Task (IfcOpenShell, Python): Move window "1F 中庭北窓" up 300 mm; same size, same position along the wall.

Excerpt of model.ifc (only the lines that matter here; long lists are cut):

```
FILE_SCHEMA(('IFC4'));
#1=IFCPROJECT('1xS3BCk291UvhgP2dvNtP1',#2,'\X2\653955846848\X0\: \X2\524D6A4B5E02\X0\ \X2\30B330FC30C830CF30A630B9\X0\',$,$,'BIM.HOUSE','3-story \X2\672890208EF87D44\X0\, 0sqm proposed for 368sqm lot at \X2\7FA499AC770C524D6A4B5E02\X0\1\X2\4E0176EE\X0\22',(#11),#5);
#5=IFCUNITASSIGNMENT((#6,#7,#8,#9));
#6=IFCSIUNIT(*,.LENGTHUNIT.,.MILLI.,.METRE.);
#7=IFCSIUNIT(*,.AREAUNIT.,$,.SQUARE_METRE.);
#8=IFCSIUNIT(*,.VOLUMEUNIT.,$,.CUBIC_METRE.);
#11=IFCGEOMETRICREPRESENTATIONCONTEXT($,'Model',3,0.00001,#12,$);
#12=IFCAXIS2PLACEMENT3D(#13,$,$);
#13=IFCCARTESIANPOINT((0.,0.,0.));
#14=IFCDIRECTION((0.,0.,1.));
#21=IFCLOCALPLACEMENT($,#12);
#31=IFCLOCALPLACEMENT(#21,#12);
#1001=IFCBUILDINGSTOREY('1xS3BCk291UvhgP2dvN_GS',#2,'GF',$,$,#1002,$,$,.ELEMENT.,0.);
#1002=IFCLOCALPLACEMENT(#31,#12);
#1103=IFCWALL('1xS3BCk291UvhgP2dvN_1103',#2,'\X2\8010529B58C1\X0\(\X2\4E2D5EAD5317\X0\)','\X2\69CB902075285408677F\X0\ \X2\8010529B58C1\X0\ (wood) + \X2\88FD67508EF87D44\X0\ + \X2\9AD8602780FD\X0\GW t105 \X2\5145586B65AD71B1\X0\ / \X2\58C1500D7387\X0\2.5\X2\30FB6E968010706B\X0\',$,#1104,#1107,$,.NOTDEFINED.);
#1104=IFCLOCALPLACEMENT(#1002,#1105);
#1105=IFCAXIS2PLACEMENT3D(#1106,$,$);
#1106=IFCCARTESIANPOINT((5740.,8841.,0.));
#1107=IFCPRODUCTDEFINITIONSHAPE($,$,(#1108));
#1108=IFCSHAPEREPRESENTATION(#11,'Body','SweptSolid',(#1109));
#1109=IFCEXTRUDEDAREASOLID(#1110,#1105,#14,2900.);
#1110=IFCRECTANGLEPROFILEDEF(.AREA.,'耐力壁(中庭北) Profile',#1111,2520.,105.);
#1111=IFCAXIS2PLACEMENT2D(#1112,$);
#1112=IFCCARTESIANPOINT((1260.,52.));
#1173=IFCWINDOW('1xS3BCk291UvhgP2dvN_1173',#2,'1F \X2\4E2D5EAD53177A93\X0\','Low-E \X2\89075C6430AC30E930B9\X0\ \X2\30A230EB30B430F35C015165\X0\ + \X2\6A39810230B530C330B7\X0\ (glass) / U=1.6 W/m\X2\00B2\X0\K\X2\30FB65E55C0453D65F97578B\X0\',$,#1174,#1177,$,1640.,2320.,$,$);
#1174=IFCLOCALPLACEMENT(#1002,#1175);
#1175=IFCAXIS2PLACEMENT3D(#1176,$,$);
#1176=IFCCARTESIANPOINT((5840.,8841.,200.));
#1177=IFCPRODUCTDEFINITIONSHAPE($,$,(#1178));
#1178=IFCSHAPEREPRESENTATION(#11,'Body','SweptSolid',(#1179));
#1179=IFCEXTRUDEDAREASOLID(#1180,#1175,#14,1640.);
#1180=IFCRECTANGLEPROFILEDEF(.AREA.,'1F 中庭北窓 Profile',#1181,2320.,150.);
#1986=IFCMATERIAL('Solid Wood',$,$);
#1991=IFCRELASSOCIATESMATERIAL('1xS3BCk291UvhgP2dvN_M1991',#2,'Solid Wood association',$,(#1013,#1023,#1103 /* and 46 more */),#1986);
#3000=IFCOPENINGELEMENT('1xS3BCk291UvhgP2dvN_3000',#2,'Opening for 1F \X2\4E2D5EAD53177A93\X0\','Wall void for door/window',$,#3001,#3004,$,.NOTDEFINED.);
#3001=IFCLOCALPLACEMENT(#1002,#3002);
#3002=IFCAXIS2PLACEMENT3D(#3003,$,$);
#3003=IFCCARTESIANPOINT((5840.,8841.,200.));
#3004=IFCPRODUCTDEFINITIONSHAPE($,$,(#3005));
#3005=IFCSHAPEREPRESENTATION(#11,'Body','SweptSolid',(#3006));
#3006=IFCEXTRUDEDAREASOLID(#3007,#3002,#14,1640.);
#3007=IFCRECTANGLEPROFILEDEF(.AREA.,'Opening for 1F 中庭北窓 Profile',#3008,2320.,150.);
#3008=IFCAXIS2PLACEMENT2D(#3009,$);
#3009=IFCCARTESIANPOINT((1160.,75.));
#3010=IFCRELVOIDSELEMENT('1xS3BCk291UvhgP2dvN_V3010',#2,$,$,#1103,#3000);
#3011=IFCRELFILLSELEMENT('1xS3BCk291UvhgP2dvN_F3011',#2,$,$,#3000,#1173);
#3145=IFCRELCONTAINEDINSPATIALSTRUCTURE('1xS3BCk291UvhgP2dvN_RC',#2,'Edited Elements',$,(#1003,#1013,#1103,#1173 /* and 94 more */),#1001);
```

```python
import numpy as np
import ifcopenshell
import ifcopenshell.api.geometry
import ifcopenshell.util.placement
import ifcopenshell.util.unit

model = ifcopenshell.open("model.ifc")
unit_scale = ifcopenshell.util.unit.calculate_unit_scale(model)

window = model.by_id(1173)
opening = window.FillsVoids[0].RelatingOpeningElement
dz = 300.0

shift = np.array([0.0, 0.0, dz])
# The window is not placed relative to its opening, so move both.
for product in (opening, window):
    matrix = ifcopenshell.util.placement.get_local_placement(product.ObjectPlacement)
    matrix[:3, 3] += shift
    ifcopenshell.api.geometry.edit_object_placement(model, product=product, matrix=matrix, is_si=False)

print(f"moved by {dz * unit_scale:+.3f} m")

model.write("model-out.ifc")
```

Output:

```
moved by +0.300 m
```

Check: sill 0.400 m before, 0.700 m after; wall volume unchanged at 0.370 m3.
